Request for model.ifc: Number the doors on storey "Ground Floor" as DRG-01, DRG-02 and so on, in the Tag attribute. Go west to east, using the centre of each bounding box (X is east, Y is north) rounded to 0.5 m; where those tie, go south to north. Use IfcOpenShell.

First a look at what the model holds.

```python
import ifcopenshell
import ifcopenshell.util.element
import ifcopenshell.util.placement

model = ifcopenshell.open("model.ifc")
print(model.schema)
storey = next(s for s in model.by_type("IfcBuildingStorey") if s.Name == "Ground Floor")
doors = [e for e in ifcopenshell.util.element.get_decomposition(storey) if e.is_a("IfcDoor")]
for e in sorted(doors, key=lambda e: e.id()):
    origin = ifcopenshell.util.placement.get_local_placement(e.ObjectPlacement)[:3, 3]
    print(e.id(), e.Tag, e.Name, origin.round(2) + 0.0, sep=" | ")
```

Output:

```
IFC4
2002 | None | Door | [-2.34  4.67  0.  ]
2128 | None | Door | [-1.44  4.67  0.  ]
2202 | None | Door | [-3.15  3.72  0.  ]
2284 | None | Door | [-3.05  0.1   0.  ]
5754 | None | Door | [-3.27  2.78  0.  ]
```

```python
import ifcopenshell
import ifcopenshell.geom
import ifcopenshell.util.element
import ifcopenshell.util.shape

model = ifcopenshell.open("model.ifc")
settings = ifcopenshell.geom.settings()
settings.set("use-world-coords", True)


def centre(element):
    shape = ifcopenshell.geom.create_shape(settings, element)
    return ifcopenshell.util.shape.get_bbox_centroid(shape.geometry)


storey = next(s for s in model.by_type("IfcBuildingStorey") if s.Name == "Ground Floor")
doors = [e for e in ifcopenshell.util.element.get_decomposition(storey) if e.is_a("IfcDoor")]

# Insertion points can sit at a corner or the storey origin, so sort by the geometry (in metres).
centres = {e: centre(e) for e in doors}
doors.sort(key=lambda e: (round(centres[e][0] / 0.5), centres[e][1]))

for i, e in enumerate(doors, start=1):
    number = f"DRG-{i:02d}"
    e.Tag = number
    print(e.id(), number)

model.write("model-out.ifc")
```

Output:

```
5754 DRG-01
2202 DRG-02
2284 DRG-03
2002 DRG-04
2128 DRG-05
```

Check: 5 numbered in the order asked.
